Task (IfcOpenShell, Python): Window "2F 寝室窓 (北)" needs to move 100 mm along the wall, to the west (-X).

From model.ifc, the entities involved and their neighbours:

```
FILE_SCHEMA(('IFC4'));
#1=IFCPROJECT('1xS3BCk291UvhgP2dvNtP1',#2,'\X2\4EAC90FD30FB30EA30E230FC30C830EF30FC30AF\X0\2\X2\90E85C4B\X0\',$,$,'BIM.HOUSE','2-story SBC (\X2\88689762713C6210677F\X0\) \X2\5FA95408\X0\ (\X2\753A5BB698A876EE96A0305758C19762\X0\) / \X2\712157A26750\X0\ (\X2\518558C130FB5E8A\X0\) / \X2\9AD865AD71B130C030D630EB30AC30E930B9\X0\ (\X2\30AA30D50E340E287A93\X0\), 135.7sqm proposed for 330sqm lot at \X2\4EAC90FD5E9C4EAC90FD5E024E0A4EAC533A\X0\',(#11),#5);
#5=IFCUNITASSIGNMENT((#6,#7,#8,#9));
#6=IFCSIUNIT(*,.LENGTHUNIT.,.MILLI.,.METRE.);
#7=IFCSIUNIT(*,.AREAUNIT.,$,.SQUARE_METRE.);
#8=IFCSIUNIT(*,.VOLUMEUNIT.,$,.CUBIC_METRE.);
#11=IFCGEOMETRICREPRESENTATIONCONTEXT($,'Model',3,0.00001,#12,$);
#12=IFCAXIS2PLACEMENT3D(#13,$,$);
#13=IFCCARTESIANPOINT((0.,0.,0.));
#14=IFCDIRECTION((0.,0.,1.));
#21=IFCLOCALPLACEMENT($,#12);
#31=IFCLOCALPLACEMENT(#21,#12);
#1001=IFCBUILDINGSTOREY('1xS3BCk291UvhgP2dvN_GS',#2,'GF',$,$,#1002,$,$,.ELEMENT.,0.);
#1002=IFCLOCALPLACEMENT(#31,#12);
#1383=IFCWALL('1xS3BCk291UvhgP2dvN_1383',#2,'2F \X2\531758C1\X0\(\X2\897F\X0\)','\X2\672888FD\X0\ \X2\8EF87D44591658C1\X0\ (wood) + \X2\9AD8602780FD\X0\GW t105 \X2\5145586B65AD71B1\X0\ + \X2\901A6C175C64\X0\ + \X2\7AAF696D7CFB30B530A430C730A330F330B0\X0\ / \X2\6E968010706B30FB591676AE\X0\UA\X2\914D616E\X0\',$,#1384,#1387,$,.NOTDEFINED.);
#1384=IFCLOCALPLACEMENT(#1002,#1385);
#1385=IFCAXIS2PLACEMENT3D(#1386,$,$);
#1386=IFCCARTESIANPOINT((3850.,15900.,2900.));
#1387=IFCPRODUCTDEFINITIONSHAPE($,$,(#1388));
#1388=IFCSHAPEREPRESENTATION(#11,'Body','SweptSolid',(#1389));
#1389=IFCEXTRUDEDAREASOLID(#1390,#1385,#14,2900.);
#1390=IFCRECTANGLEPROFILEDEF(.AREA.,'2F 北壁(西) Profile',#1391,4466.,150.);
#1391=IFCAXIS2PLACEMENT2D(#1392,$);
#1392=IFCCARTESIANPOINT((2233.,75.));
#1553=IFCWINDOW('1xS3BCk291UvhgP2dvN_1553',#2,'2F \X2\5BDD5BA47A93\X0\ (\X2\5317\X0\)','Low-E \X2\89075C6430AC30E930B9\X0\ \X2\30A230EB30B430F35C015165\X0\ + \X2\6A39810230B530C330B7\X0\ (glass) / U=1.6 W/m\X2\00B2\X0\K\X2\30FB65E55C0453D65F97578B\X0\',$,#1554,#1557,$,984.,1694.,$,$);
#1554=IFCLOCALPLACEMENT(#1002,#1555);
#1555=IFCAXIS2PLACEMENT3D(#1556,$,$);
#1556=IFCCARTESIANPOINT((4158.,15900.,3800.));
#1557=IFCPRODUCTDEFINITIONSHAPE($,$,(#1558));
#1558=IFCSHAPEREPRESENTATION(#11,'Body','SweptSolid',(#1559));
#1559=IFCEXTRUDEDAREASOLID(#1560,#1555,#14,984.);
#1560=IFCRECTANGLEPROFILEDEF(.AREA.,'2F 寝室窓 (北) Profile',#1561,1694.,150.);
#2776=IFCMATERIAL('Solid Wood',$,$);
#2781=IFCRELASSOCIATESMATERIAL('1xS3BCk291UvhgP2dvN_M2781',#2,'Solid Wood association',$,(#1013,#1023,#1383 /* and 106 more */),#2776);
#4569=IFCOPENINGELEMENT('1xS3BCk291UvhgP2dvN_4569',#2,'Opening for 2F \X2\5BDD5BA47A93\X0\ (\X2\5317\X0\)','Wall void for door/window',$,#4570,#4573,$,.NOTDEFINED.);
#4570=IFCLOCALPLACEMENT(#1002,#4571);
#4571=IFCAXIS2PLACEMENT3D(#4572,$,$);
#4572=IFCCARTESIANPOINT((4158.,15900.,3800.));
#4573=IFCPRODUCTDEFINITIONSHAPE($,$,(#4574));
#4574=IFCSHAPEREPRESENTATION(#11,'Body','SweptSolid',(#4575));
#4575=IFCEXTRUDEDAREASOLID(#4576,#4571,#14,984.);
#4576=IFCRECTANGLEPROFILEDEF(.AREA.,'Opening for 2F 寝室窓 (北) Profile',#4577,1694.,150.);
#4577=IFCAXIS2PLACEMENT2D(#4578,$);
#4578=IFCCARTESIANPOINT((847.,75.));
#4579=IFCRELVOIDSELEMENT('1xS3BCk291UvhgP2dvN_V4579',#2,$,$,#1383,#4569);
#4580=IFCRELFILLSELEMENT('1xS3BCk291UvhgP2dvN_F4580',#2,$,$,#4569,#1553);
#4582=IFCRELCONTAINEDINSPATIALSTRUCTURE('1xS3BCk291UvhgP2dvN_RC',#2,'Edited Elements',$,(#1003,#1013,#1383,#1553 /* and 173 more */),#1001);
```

```python
import ifcopenshell
import ifcopenshell.api.geometry
import ifcopenshell.util.placement
import ifcopenshell.util.unit

model = ifcopenshell.open("model.ifc")
unit_scale = ifcopenshell.util.unit.calculate_unit_scale(model)

window = model.by_guid("1xS3BCk291UvhgP2dvN_1553")
opening = window.FillsVoids[0].RelatingOpeningElement
wall = opening.VoidsElements[0].RelatingBuildingElement

wall_matrix = ifcopenshell.util.placement.get_local_placement(wall.ObjectPlacement)
shift = wall_matrix[:3, 0] * -0.1 / unit_scale
before = ifcopenshell.util.placement.get_local_placement(window.ObjectPlacement)[:3, 3].copy()

# The window is not placed relative to its opening, so move both.
for product in (opening, window):
    matrix = ifcopenshell.util.placement.get_local_placement(product.ObjectPlacement)
    matrix[:3, 3] += shift
    ifcopenshell.api.geometry.edit_object_placement(model, product=product, matrix=matrix, is_si=False)

after = ifcopenshell.util.placement.get_local_placement(window.ObjectPlacement)[:3, 3]
print("window moved by", (after - before).round(3) + 0.0)

model.write("model_rev.ifc")
```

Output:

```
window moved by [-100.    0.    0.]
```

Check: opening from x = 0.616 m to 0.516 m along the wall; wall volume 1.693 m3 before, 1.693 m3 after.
